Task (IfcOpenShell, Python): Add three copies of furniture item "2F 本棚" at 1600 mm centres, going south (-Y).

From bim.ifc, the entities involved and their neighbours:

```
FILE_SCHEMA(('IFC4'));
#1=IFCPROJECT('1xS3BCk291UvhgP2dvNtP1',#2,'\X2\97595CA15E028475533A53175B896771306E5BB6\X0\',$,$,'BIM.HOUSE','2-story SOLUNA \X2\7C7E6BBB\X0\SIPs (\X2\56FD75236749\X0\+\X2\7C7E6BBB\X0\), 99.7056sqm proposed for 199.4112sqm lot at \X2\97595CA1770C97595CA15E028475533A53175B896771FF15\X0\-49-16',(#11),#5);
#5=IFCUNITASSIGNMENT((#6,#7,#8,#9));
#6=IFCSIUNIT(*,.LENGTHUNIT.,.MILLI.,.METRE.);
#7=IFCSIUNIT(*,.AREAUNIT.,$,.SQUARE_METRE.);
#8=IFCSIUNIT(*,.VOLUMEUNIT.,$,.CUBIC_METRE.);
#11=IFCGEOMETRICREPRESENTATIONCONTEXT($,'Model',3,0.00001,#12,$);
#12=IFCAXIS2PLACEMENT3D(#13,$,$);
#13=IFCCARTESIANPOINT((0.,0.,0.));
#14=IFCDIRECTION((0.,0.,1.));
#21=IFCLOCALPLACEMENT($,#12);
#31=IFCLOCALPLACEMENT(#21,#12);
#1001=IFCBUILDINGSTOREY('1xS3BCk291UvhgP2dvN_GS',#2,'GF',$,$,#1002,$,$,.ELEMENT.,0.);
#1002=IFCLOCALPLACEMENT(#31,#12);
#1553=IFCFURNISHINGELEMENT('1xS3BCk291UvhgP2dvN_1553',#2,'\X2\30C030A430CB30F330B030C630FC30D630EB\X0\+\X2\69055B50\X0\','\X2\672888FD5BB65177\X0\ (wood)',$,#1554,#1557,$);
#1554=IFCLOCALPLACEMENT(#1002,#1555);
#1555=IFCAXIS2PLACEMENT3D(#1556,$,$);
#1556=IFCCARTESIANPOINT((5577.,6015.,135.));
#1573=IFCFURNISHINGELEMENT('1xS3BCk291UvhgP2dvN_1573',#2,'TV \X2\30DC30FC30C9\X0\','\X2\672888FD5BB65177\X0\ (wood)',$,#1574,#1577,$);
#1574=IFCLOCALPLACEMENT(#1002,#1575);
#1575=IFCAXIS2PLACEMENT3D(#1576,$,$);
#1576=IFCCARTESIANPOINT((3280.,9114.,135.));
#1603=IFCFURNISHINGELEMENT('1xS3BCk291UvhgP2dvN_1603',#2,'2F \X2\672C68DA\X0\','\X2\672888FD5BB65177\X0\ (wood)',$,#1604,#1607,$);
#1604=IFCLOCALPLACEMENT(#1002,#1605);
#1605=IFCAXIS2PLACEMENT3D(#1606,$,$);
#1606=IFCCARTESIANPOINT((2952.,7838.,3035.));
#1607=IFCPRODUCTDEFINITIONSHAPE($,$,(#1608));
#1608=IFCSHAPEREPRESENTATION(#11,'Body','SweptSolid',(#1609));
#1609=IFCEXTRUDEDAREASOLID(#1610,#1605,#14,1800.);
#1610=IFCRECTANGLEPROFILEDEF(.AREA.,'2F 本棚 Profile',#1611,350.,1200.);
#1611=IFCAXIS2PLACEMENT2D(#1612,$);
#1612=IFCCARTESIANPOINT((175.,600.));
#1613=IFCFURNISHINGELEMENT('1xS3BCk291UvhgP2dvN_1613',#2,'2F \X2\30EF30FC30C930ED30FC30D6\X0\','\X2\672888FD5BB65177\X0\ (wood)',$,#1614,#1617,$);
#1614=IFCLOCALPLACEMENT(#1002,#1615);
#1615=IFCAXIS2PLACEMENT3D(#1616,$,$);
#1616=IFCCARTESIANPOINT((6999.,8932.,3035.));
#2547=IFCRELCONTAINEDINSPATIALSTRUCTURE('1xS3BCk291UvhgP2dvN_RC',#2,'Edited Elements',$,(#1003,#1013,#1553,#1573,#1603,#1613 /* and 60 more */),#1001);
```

```python
import numpy as np
import ifcopenshell
import ifcopenshell.api.geometry
import ifcopenshell.api.root
import ifcopenshell.util.element
import ifcopenshell.util.placement
import ifcopenshell.util.unit

model = ifcopenshell.open("bim.ifc")
unit_scale = ifcopenshell.util.unit.calculate_unit_scale(model)


def reuse_history(source, copy):
    """copy_class also copies each property set's owner history, people and application; keep the originals."""
    for rel in copy.IsDefinedBy:
        if rel.is_a("IfcRelDefinesByProperties") and (history := rel.RelatingPropertyDefinition.OwnerHistory):
            rel.RelatingPropertyDefinition.OwnerHistory = source.OwnerHistory
            ifcopenshell.util.element.remove_deep2(model, history)


source = model.by_guid("1xS3BCk291UvhgP2dvN_1603")
base = ifcopenshell.util.placement.get_local_placement(source.ObjectPlacement)
step = np.array([0.0, -1.0, 0.0]) * 1.6 / unit_scale

for i in range(1, 4):
    copy = ifcopenshell.api.root.copy_class(model, product=source)
    copy.Representation = ifcopenshell.util.element.copy_deep(
        model, source.Representation, exclude=["IfcGeometricRepresentationContext", "IfcRepresentationMap"]
    )
    reuse_history(source, copy)
    matrix = base.copy()
    matrix[:3, 3] += i * step
    print("added at", matrix[:3, 3].round(3) + 0.0)
    ifcopenshell.api.geometry.edit_object_placement(model, product=copy, matrix=matrix, is_si=False)

model.write("bim_updated.ifc")
```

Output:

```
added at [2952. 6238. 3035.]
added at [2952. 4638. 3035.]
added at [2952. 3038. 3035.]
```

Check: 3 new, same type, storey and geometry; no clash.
